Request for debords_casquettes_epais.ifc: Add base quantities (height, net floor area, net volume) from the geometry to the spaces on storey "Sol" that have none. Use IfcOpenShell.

First a look at what the model holds.

```python
import ifcopenshell
import ifcopenshell.util.element
import ifcopenshell.util.unit

model = ifcopenshell.open("debords_casquettes_epais.ifc")
print(model.schema)
for unit_type in ("LENGTHUNIT", "AREAUNIT", "VOLUMEUNIT"):
    print(unit_type, ifcopenshell.util.unit.calculate_unit_scale(model, unit_type))
storey = next(s for s in model.by_type("IfcBuildingStorey") if s.Name == "Sol")
spaces = [e for e in ifcopenshell.util.element.get_decomposition(storey) if e.is_a("IfcSpace")]
for e in sorted(spaces, key=lambda e: e.id()):
    print(e.id(), e.is_a(), e.Name, list(ifcopenshell.util.element.get_psets(e, qtos_only=True)), sep=" | ")
```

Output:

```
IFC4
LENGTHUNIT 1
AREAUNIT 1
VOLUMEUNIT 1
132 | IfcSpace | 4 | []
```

```python
import ifcopenshell
import ifcopenshell.api.pset
import ifcopenshell.geom
import ifcopenshell.util.element
import ifcopenshell.util.shape
import ifcopenshell.util.unit

model = ifcopenshell.open("debords_casquettes_epais.ifc")
unit_scale = ifcopenshell.util.unit.calculate_unit_scale(model)
area_scale = ifcopenshell.util.unit.calculate_unit_scale(model, "AREAUNIT")
volume_scale = ifcopenshell.util.unit.calculate_unit_scale(model, "VOLUMEUNIT")
settings = ifcopenshell.geom.settings()

storey = next(s for s in model.by_type("IfcBuildingStorey") if s.Name == "Sol")
spaces = [e for e in ifcopenshell.util.element.get_decomposition(storey) if e.is_a("IfcSpace")]

for e in sorted(spaces, key=lambda e: e.id()):
    if ifcopenshell.util.element.get_psets(e, qtos_only=True, should_inherit=False):
        continue
    # Geometry comes back in metres, in the element's own axes.
    shape = ifcopenshell.geom.create_shape(settings, e)
    values = {
        "Height": ifcopenshell.util.shape.get_z(shape.geometry) / unit_scale,
        "NetFloorArea": ifcopenshell.util.shape.get_footprint_area(shape.geometry) / area_scale,
        "NetVolume": ifcopenshell.util.shape.get_volume(shape.geometry) / volume_scale,
    }
    qto = ifcopenshell.api.pset.add_qto(model, product=e, name="Qto_SpaceBaseQuantities")
    ifcopenshell.api.pset.edit_qto(model, qto=qto, properties=values)
    print(e.id(), {k: round(v, 3) for k, v in values.items()})

model.write("debords_casquettes_epais_updated.ifc")
```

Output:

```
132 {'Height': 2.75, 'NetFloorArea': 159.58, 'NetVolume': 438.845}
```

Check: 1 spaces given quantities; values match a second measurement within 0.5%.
